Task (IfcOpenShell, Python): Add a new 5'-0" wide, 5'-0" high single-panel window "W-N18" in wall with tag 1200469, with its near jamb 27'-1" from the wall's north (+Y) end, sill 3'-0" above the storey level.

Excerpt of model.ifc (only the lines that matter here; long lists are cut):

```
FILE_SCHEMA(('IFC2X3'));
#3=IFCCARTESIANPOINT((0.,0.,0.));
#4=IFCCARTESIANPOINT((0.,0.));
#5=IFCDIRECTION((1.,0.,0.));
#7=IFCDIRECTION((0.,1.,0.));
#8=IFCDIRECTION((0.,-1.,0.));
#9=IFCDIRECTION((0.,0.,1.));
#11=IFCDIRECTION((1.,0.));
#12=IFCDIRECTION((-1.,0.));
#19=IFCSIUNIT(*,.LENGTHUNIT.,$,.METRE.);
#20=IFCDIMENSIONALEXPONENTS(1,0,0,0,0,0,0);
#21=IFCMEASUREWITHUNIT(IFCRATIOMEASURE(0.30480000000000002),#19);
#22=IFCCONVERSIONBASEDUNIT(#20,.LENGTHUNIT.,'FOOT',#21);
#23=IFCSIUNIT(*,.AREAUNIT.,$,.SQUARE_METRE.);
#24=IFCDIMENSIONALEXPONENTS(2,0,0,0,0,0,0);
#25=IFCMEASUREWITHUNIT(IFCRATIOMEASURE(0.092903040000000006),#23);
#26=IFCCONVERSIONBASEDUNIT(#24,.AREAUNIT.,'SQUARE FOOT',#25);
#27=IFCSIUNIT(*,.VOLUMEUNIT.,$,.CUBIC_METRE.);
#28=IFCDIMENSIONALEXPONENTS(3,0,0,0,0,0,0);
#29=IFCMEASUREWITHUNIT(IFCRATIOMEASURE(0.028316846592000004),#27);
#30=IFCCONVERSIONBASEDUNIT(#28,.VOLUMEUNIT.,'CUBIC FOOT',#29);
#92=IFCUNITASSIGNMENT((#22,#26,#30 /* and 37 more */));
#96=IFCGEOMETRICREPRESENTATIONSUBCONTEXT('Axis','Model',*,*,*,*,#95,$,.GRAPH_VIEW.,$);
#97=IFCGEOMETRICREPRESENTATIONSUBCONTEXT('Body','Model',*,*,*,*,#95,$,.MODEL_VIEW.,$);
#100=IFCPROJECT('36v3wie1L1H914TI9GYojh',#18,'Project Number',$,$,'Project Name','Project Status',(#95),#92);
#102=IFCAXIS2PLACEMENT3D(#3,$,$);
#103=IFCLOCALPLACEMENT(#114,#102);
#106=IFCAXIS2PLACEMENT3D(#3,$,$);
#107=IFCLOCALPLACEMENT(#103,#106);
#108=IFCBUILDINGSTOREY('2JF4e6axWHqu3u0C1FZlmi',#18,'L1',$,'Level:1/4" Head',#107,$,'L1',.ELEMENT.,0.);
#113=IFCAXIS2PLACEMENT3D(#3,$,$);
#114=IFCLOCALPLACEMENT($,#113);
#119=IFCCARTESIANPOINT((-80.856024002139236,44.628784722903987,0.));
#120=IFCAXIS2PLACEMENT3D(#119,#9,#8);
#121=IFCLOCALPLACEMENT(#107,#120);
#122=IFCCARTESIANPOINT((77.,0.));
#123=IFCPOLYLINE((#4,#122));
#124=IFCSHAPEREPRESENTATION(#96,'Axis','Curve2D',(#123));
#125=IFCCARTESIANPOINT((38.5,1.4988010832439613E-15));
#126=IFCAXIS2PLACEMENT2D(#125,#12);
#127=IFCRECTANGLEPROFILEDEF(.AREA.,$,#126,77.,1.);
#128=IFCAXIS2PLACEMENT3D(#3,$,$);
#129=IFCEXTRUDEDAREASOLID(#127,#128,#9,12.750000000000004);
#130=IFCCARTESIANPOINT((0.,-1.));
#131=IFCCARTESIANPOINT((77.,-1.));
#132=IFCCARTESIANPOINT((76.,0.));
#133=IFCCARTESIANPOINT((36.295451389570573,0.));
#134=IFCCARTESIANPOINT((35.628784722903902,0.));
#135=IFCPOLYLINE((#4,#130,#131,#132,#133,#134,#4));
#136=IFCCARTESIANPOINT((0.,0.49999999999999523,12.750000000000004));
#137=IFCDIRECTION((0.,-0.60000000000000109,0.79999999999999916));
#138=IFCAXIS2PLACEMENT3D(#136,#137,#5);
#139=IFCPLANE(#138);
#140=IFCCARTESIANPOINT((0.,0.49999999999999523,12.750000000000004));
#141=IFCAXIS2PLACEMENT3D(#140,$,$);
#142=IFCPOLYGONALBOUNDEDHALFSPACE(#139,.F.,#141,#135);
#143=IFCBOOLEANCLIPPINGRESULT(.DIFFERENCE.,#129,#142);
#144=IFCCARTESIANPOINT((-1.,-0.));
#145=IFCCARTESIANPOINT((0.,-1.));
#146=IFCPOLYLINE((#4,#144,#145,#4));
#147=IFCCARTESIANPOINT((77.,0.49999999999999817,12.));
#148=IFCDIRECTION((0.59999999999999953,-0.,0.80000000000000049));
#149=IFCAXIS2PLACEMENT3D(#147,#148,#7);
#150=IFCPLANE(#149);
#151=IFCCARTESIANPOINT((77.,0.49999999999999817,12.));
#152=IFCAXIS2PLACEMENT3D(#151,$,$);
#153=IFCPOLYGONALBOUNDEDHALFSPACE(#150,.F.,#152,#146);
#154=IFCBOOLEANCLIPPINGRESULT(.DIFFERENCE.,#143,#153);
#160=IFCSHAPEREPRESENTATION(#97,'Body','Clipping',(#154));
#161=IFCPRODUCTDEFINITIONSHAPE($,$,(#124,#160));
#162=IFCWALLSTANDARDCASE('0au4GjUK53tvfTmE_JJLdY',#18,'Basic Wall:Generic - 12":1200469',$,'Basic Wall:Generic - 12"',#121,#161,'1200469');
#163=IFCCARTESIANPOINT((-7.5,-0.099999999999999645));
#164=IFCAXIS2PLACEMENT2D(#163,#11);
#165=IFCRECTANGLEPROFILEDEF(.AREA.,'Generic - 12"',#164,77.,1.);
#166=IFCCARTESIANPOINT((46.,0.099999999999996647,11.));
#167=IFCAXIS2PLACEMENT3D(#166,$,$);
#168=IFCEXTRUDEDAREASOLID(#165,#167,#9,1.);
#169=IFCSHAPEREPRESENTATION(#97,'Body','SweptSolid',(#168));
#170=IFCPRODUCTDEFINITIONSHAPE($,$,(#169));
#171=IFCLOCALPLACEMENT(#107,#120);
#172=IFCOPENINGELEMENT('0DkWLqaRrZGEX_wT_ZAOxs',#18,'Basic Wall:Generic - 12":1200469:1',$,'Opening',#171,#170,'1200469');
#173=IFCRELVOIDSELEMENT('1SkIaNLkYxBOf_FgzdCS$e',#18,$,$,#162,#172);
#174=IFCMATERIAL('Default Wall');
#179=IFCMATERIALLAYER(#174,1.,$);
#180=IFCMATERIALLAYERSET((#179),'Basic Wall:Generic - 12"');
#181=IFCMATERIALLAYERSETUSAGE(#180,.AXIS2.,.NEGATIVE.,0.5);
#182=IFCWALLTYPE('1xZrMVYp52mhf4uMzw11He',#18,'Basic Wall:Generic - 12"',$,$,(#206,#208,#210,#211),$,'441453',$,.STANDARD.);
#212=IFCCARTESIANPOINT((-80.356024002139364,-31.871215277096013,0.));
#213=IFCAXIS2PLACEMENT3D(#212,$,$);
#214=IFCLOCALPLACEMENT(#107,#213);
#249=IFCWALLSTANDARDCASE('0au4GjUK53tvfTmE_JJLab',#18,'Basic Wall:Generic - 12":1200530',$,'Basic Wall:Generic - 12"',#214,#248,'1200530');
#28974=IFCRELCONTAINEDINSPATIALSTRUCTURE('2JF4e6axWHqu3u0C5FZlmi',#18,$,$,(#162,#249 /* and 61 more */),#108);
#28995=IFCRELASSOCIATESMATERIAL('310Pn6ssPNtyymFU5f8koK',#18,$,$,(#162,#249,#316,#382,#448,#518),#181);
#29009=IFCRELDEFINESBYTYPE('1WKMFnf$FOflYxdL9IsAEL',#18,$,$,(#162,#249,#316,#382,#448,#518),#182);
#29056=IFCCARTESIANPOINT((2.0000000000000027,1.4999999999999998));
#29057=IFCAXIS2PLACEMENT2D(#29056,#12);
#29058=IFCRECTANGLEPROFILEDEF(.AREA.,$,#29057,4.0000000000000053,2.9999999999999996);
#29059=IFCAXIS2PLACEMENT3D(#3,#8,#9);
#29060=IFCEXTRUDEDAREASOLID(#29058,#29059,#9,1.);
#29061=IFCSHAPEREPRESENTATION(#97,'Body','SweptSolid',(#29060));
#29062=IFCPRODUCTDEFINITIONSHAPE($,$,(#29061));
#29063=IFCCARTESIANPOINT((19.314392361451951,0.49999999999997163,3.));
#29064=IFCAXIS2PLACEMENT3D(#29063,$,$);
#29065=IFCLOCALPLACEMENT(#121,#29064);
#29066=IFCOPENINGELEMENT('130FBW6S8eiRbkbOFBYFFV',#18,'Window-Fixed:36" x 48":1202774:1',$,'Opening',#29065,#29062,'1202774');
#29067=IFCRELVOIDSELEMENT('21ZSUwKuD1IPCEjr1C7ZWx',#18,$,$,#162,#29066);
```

```python
import numpy as np
import ifcopenshell
import ifcopenshell.api.feature
import ifcopenshell.api.geometry
import ifcopenshell.api.root
import ifcopenshell.api.spatial
import ifcopenshell.api.type
import ifcopenshell.geom
import ifcopenshell.util.element
import ifcopenshell.util.placement
import ifcopenshell.util.representation
import ifcopenshell.util.shape
import ifcopenshell.util.unit

model = ifcopenshell.open("model.ifc")
unit_scale = ifcopenshell.util.unit.calculate_unit_scale(model)
settings = ifcopenshell.geom.settings()


def volume(element):
    """Net volume in cubic metres, openings subtracted."""
    shape = ifcopenshell.geom.create_shape(settings, element)
    return ifcopenshell.util.shape.get_volume(shape.geometry)


wall = model.by_guid("0au4GjUK53tvfTmE_JJLdY")
storey = ifcopenshell.util.element.get_container(wall, ifc_class="IfcBuildingStorey")
context = ifcopenshell.util.representation.get_context(model, "Model", "Body", "MODEL_VIEW")
before = volume(wall)

width, height, from_end, sill = 1.524, 1.524, 8.255, 0.9144  # metres

# The wall runs along its own X axis, and the end named is its -X end.
wall_shape = ifcopenshell.geom.create_shape(settings, wall)
x, y, z = ifcopenshell.util.shape.get_vertices(wall_shape.geometry).T
start = x.min() + from_end
face, thickness = float(y.min()), float(y.max() - y.min())
wall_matrix = ifcopenshell.util.placement.get_local_placement(wall.ObjectPlacement)
level = ifcopenshell.util.placement.get_local_placement(storey.ObjectPlacement)[2, 3]


def in_wall(x, y):
    """Placement at x, y metres in the wall's axes, at sill height."""
    matrix = wall_matrix.copy()
    matrix[:, 3] = wall_matrix @ np.array([x / unit_scale, y / unit_scale, 0.0, 1.0])
    matrix[2, 3] = level + sill / unit_scale
    return matrix


# Opening: a box that overshoots both wall faces by 50 mm.
opening = ifcopenshell.api.root.create_entity(model, ifc_class="IfcOpeningElement")
box = ifcopenshell.api.geometry.add_wall_representation(
    model, context=context, length=width, height=height, thickness=thickness + 0.1
)
ifcopenshell.api.geometry.assign_representation(model, product=opening, representation=box)
ifcopenshell.api.geometry.edit_object_placement(model, product=opening, matrix=in_wall(start, face - 0.05), is_si=False)
ifcopenshell.api.feature.add_feature(model, feature=opening, element=wall)

window = ifcopenshell.api.root.create_entity(model, ifc_class="IfcWindow", name="W-N18")
window.OverallWidth, window.OverallHeight = width / unit_scale, height / unit_scale
body = ifcopenshell.api.geometry.add_window_representation(
    model,
    context=context,
    overall_width=window.OverallWidth,
    overall_height=window.OverallHeight,
    partition_type="SINGLE_PANEL",
)
ifcopenshell.api.geometry.assign_representation(model, product=window, representation=body)
ifcopenshell.api.spatial.assign_container(model, products=[window], relating_structure=storey)
fills = ifcopenshell.api.feature.add_filling(model, opening=opening, element=window)
fills.OwnerHistory = window.OwnerHistory  # required in IFC2X3

# IFC2X3 keeps the operation on the window style.
style = ifcopenshell.api.root.create_entity(model, ifc_class="IfcWindowStyle", name="W-N18")
style.OperationType, style.ConstructionType = "SINGLE_PANEL", "NOTDEFINED"
style.ParameterTakesPrecedence = style.Sizeable = False
ifcopenshell.api.type.assign_type(model, related_objects=[window], relating_type=style)

# Centre the window in the wall's thickness.
ifcopenshell.api.geometry.edit_object_placement(model, product=window, matrix=in_wall(start, face), is_si=False)
window_shape = ifcopenshell.geom.create_shape(settings, window)
depth = ifcopenshell.util.shape.get_vertices(window_shape.geometry)[:, 1]
offset = face + thickness / 2 - (depth.min() + depth.max()) / 2
ifcopenshell.api.geometry.edit_object_placement(model, product=window, matrix=in_wall(start, offset), is_si=False)

after = volume(wall)

print(f"wall volume {before:.3f} -> {after:.3f} m3")

model.write("model-out.ifc")
```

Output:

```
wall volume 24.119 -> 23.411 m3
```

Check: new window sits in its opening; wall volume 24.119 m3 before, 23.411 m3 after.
